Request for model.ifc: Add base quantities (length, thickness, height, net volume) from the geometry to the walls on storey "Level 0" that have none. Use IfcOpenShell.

First a look at what the model holds.

```python
import ifcopenshell
import ifcopenshell.util.element
import ifcopenshell.util.unit

model = ifcopenshell.open("model.ifc")
print(model.schema)
for unit_type in ("LENGTHUNIT", "AREAUNIT", "VOLUMEUNIT"):
    print(unit_type, ifcopenshell.util.unit.calculate_unit_scale(model, unit_type))
storey = next(s for s in model.by_type("IfcBuildingStorey") if s.Name == "Level 0")
walls = [e for e in ifcopenshell.util.element.get_decomposition(storey) if e.is_a("IfcWall")]
for e in sorted(walls, key=lambda e: e.id()):
    print(e.id(), e.is_a(), e.Name, list(ifcopenshell.util.element.get_psets(e, qtos_only=True)), sep=" | ")
```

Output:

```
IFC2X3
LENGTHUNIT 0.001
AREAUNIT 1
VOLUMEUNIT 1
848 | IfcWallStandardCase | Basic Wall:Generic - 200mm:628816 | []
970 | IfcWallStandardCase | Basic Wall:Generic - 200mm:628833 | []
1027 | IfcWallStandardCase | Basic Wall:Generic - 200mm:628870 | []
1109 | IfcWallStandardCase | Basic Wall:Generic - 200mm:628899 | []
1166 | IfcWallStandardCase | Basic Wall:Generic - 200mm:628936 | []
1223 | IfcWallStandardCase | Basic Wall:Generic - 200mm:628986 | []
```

```python
import ifcopenshell
import ifcopenshell.api.pset
import ifcopenshell.geom
import ifcopenshell.util.element
import ifcopenshell.util.shape
import ifcopenshell.util.unit

model = ifcopenshell.open("model.ifc")
unit_scale = ifcopenshell.util.unit.calculate_unit_scale(model)
volume_scale = ifcopenshell.util.unit.calculate_unit_scale(model, "VOLUMEUNIT")
settings = ifcopenshell.geom.settings()

storey = next(s for s in model.by_type("IfcBuildingStorey") if s.Name == "Level 0")
walls = [e for e in ifcopenshell.util.element.get_decomposition(storey) if e.is_a("IfcWall")]

for e in sorted(walls, key=lambda e: e.id()):
    if ifcopenshell.util.element.get_psets(e, qtos_only=True, should_inherit=False):
        continue
    # Geometry comes back in metres, in the element's own axes.
    shape = ifcopenshell.geom.create_shape(settings, e)
    values = {
        "Length": ifcopenshell.util.shape.get_x(shape.geometry) / unit_scale,
        "Width": ifcopenshell.util.shape.get_y(shape.geometry) / unit_scale,
        "Height": ifcopenshell.util.shape.get_z(shape.geometry) / unit_scale,
        "NetVolume": ifcopenshell.util.shape.get_volume(shape.geometry) / volume_scale,
    }
    qto = ifcopenshell.api.pset.add_qto(model, product=e, name="BaseQuantities")
    ifcopenshell.api.pset.edit_qto(model, qto=qto, properties=values)
    print(e.id(), {k: round(v, 3) for k, v in values.items()})

model.write("model-out.ifc")
```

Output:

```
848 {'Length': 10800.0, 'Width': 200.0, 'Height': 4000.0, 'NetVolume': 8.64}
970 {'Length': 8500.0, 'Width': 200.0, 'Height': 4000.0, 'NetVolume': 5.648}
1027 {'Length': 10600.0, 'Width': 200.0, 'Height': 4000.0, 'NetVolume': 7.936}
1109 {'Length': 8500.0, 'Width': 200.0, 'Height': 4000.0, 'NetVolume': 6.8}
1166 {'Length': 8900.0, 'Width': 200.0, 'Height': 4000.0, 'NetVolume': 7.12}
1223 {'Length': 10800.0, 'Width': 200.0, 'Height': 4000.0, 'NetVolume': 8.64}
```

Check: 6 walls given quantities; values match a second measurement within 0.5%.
